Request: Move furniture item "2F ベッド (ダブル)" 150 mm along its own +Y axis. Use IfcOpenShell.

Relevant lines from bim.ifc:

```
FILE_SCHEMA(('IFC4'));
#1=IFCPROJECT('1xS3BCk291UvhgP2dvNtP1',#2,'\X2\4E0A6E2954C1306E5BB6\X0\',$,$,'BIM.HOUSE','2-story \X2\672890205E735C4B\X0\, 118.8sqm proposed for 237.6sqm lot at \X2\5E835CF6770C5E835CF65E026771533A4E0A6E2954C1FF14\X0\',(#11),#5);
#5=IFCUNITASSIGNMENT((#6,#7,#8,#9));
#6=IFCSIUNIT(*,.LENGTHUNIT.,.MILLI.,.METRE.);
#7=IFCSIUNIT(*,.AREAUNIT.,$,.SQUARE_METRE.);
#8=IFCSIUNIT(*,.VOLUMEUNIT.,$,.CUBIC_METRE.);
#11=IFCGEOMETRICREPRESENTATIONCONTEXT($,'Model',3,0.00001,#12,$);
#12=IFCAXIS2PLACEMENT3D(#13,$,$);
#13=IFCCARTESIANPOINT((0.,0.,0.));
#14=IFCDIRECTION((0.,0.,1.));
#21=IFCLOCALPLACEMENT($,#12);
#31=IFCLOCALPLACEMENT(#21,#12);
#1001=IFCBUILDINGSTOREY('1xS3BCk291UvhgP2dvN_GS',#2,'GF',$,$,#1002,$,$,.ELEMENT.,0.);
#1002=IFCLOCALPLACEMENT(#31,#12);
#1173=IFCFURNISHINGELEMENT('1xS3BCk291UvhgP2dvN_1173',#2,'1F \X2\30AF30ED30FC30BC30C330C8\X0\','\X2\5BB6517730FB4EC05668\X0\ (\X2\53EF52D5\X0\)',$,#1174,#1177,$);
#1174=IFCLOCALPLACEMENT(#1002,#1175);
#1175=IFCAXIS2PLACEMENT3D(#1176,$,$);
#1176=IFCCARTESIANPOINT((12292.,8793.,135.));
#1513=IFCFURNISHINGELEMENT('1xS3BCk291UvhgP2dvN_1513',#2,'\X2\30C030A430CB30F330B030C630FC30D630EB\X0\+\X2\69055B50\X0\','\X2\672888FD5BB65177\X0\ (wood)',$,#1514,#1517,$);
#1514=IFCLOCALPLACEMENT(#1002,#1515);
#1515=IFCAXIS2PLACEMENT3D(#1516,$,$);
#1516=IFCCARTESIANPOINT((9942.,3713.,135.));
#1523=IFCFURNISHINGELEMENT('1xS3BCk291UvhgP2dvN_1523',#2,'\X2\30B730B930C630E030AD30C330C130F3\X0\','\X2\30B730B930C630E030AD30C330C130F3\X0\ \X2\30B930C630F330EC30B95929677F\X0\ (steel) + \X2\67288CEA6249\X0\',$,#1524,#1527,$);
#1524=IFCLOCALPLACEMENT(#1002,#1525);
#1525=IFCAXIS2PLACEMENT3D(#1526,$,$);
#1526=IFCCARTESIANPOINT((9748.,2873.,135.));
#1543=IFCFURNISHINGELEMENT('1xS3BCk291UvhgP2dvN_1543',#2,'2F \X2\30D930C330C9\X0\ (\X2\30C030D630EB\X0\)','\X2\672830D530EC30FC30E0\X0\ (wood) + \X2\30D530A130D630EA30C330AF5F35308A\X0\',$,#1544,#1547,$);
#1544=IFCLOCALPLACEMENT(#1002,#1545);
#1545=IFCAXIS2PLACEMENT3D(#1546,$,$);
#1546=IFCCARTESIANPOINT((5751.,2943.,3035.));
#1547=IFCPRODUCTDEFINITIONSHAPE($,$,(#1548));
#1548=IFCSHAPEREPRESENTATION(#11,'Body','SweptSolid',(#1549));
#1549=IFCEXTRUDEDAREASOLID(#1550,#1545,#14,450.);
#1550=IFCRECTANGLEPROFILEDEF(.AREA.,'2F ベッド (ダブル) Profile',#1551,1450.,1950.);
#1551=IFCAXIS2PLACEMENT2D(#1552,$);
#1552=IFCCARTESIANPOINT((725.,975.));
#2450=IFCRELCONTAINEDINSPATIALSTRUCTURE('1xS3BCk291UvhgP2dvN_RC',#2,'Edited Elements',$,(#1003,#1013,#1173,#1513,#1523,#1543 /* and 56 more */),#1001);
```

```python
import ifcopenshell
import ifcopenshell.api.geometry
import ifcopenshell.util.placement
import ifcopenshell.util.unit

model = ifcopenshell.open("bim.ifc")
unit_scale = ifcopenshell.util.unit.calculate_unit_scale(model)

item = model.by_guid("1xS3BCk291UvhgP2dvN_1543")
matrix = ifcopenshell.util.placement.get_local_placement(item.ObjectPlacement)
matrix[:3, 3] += matrix[:3, 1] * 0.15 / unit_scale
ifcopenshell.api.geometry.edit_object_placement(model, product=item, matrix=matrix, is_si=False)

print(ifcopenshell.util.placement.get_local_placement(item.ObjectPlacement).round(3) + 0.0)

model.write("bim_v2.ifc")
```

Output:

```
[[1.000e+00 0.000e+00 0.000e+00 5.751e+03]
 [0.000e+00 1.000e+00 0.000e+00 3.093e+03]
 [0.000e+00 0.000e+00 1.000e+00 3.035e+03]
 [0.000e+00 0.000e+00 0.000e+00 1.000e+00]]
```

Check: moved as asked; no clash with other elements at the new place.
